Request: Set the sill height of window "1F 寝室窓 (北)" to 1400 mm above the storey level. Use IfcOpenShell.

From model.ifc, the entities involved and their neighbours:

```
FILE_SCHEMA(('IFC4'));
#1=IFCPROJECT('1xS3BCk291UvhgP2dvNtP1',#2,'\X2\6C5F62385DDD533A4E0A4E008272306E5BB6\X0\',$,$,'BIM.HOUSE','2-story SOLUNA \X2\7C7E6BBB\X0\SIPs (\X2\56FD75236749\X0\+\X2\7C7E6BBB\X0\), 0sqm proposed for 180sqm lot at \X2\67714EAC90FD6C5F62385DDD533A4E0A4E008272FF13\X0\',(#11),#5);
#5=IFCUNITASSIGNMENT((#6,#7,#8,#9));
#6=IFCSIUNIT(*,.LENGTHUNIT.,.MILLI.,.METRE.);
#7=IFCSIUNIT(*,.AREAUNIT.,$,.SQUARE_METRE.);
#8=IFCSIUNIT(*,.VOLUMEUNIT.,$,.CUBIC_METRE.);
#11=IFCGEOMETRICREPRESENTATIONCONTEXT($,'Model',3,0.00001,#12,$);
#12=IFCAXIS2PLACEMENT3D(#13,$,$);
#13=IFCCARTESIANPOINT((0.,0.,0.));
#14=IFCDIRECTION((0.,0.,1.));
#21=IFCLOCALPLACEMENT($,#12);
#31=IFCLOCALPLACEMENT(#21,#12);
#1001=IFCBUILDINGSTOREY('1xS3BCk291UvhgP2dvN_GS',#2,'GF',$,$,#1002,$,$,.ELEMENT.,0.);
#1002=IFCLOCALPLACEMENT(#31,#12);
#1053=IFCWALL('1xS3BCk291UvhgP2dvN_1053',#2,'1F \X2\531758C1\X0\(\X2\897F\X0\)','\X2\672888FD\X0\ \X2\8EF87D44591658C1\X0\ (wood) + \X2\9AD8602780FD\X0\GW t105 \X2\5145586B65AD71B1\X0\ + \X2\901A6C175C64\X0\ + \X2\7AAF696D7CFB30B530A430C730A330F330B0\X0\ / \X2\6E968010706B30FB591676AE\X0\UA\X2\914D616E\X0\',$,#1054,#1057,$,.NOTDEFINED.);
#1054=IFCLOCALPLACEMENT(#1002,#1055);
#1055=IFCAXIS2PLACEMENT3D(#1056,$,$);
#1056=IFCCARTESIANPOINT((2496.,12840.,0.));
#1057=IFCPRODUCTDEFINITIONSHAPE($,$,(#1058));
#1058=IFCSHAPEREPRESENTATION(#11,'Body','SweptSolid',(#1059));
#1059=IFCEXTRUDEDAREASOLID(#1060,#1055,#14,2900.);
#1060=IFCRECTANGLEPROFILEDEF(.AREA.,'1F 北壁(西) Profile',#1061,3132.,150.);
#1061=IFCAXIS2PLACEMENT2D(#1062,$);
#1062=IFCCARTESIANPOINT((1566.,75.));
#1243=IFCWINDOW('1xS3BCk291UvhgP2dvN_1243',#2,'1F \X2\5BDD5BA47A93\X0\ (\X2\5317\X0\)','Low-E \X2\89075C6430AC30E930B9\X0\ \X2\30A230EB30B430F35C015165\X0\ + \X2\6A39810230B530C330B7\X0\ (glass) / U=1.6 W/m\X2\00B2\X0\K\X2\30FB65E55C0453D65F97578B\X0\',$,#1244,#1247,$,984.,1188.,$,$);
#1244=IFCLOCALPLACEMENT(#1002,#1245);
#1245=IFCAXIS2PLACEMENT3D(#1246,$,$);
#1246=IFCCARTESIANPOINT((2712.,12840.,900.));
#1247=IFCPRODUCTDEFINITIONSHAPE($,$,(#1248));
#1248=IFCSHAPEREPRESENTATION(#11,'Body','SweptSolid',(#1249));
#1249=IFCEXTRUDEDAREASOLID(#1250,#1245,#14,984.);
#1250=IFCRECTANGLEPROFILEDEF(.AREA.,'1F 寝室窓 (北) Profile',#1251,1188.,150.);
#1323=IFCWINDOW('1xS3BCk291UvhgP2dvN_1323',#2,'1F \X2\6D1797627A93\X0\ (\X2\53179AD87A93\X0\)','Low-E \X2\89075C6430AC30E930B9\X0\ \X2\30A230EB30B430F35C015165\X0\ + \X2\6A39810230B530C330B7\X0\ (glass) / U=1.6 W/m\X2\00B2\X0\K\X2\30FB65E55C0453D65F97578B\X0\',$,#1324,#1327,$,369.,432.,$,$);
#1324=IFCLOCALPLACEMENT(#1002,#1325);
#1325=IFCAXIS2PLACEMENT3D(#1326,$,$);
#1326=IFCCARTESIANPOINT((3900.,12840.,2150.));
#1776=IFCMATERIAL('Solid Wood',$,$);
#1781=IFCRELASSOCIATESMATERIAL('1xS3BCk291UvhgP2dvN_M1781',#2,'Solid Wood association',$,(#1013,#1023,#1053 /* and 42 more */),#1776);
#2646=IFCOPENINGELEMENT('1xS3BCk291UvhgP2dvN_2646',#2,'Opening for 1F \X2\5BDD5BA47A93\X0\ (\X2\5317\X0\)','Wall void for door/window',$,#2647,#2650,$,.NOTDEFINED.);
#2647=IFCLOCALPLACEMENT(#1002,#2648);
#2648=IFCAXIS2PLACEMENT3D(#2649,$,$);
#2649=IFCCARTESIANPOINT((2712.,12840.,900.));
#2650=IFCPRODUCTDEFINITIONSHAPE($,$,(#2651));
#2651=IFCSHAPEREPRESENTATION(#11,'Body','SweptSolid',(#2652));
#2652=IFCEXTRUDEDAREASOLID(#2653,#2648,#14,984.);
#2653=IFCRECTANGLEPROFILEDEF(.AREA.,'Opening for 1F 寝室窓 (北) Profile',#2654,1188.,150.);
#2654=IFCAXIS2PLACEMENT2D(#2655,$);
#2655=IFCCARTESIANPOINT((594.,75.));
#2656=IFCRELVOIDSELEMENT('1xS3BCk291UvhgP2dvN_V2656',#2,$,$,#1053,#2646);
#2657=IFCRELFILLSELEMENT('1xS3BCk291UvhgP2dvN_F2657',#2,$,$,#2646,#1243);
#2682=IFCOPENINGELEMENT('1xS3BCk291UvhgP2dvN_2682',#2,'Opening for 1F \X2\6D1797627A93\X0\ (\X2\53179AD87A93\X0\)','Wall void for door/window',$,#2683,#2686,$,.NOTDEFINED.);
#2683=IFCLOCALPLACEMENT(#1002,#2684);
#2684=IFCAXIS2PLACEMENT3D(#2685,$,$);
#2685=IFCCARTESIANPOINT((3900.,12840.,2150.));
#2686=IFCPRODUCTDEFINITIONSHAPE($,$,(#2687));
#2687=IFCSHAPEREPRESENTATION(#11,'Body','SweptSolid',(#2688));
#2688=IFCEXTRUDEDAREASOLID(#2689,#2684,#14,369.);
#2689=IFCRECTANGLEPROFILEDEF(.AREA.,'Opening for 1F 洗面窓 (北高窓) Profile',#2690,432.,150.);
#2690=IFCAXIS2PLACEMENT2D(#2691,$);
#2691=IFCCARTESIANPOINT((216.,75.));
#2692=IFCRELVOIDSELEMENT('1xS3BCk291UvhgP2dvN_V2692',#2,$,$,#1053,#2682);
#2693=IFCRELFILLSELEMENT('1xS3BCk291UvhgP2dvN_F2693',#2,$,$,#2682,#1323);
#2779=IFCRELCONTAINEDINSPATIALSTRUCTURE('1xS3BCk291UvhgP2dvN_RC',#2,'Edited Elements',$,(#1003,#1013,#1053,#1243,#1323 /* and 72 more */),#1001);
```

```python
import numpy as np
import ifcopenshell
import ifcopenshell.api.geometry
import ifcopenshell.geom
import ifcopenshell.util.element
import ifcopenshell.util.placement
import ifcopenshell.util.shape
import ifcopenshell.util.unit

model = ifcopenshell.open("model.ifc")
unit_scale = ifcopenshell.util.unit.calculate_unit_scale(model)

window = model.by_id(1243)
opening = window.FillsVoids[0].RelatingOpeningElement
storey = ifcopenshell.util.element.get_container(window, ifc_class="IfcBuildingStorey")
level = ifcopenshell.util.placement.get_local_placement(storey.ObjectPlacement)[2, 3]

# The opening's origin need not be at the sill, so measure its lowest point.
shape = ifcopenshell.geom.create_shape(ifcopenshell.geom.settings(), opening)
bottom = ifcopenshell.util.shape.get_shape_bottom_elevation(shape, shape.geometry) / unit_scale
dz = level + 1400.0 - bottom

shift = np.array([0.0, 0.0, dz])
# The window is not placed relative to its opening, so move both.
for product in (opening, window):
    matrix = ifcopenshell.util.placement.get_local_placement(product.ObjectPlacement)
    matrix[:3, 3] += shift
    ifcopenshell.api.geometry.edit_object_placement(model, product=product, matrix=matrix, is_si=False)

print(f"moved by {dz * unit_scale:+.3f} m")

model.write("model_edited.ifc")
```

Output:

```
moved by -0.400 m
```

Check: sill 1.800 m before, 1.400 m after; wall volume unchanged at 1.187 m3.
